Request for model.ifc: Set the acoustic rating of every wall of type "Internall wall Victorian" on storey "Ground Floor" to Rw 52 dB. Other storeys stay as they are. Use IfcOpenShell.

First a look at what the model holds.

```python
import ifcopenshell
import ifcopenshell.util.element

model = ifcopenshell.open("model.ifc")
print(model.schema)
storey = next(s for s in model.by_type("IfcBuildingStorey") if s.Name == "Ground Floor")
walls = [e for e in ifcopenshell.util.element.get_decomposition(storey) if e.is_a("IfcWall")]
seen = {}
for e in walls:
    element_type = ifcopenshell.util.element.get_type(e)
    key = (element_type.Name if element_type != e and element_type else None, ifcopenshell.util.element.get_pset(e, "Pset_WallCommon", "AcousticRating"))
    seen[key] = seen.get(key, 0) + 1
for (name, value), count in sorted(seen.items(), key=str):
    print(count, "x", name, "|", value)
```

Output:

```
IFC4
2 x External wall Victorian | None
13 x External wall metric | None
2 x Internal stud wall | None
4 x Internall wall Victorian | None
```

```python
import ifcopenshell
import ifcopenshell.api.pset
import ifcopenshell.util.element

model = ifcopenshell.open("model.ifc")

storey = next(s for s in model.by_type("IfcBuildingStorey") if s.Name == "Ground Floor")
walls = [e for e in ifcopenshell.util.element.get_decomposition(storey) if e.is_a("IfcWall")]

count = 0
for e in walls:
    element_type = ifcopenshell.util.element.get_type(e)
    if element_type in (None, e) or element_type.Name != "Internall wall Victorian":
        continue
    # add_pset returns the element's existing set when there is one.
    pset = ifcopenshell.api.pset.add_pset(model, product=e, name="Pset_WallCommon")
    ifcopenshell.api.pset.edit_pset(model, pset=pset, properties={"AcousticRating": "Rw 52 dB"})
    count += 1

print(count, "walls updated")

model.write("model_edited.ifc")
```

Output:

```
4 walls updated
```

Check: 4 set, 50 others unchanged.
